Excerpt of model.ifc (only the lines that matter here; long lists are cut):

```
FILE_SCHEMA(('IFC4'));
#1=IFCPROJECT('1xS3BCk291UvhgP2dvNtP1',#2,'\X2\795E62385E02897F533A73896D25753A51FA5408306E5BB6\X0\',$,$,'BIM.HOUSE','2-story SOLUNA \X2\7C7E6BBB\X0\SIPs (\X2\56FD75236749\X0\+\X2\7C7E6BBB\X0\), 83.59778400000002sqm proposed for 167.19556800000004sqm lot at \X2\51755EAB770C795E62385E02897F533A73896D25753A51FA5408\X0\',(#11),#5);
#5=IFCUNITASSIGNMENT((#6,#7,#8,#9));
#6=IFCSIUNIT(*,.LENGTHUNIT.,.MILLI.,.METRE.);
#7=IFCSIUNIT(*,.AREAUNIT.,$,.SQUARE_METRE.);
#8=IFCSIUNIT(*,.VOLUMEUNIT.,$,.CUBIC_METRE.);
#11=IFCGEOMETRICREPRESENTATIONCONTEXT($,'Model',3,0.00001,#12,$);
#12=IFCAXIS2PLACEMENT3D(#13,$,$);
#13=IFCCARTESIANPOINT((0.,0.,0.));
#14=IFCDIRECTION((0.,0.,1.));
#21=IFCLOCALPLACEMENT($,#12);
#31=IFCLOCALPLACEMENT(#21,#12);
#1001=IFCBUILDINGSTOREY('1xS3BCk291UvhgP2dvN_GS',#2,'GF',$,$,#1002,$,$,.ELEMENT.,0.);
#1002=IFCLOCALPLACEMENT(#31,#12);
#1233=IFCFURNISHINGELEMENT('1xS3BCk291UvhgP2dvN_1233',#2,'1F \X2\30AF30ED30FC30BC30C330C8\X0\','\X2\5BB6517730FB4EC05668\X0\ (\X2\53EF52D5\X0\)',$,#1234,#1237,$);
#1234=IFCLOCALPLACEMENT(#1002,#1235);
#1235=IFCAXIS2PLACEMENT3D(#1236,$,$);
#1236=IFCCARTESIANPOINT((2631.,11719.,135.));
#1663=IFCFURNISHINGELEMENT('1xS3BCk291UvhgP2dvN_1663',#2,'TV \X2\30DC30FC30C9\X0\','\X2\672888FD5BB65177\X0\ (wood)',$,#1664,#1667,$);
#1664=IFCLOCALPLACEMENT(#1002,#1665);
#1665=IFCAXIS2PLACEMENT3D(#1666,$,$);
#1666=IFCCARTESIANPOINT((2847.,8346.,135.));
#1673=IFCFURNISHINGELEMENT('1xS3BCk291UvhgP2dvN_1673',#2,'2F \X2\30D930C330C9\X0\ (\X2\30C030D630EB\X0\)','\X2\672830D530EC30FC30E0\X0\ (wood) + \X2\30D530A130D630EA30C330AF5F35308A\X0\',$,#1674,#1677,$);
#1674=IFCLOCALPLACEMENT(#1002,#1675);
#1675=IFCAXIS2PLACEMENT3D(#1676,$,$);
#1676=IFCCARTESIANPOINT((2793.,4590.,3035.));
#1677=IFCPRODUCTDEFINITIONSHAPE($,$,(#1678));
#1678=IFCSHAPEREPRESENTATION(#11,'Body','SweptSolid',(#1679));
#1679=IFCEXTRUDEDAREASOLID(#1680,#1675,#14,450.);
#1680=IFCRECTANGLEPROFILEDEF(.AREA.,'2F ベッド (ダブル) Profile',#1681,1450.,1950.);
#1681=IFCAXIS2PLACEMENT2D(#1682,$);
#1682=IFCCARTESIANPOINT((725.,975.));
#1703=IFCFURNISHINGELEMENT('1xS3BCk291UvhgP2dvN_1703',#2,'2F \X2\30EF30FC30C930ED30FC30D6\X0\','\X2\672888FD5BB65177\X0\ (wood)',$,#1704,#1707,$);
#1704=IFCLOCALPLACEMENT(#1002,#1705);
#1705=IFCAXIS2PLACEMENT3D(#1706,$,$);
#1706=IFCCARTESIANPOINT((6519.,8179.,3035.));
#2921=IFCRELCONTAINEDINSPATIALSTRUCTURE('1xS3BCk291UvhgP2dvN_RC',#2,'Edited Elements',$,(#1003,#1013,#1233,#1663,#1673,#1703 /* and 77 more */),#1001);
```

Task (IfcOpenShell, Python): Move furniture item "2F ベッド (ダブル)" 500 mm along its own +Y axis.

```python
import ifcopenshell
import ifcopenshell.api.geometry
import ifcopenshell.util.placement
import ifcopenshell.util.unit

model = ifcopenshell.open("model.ifc")
unit_scale = ifcopenshell.util.unit.calculate_unit_scale(model)

item = model.by_guid("1xS3BCk291UvhgP2dvN_1673")
matrix = ifcopenshell.util.placement.get_local_placement(item.ObjectPlacement)
matrix[:3, 3] += matrix[:3, 1] * 0.5 / unit_scale
ifcopenshell.api.geometry.edit_object_placement(model, product=item, matrix=matrix, is_si=False)

print(ifcopenshell.util.placement.get_local_placement(item.ObjectPlacement).round(3) + 0.0)

model.write("model_updated.ifc")
```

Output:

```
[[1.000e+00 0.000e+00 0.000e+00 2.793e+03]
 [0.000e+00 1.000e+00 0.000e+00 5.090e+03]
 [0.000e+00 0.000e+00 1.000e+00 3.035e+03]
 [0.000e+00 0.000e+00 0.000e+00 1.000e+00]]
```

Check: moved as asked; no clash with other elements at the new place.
